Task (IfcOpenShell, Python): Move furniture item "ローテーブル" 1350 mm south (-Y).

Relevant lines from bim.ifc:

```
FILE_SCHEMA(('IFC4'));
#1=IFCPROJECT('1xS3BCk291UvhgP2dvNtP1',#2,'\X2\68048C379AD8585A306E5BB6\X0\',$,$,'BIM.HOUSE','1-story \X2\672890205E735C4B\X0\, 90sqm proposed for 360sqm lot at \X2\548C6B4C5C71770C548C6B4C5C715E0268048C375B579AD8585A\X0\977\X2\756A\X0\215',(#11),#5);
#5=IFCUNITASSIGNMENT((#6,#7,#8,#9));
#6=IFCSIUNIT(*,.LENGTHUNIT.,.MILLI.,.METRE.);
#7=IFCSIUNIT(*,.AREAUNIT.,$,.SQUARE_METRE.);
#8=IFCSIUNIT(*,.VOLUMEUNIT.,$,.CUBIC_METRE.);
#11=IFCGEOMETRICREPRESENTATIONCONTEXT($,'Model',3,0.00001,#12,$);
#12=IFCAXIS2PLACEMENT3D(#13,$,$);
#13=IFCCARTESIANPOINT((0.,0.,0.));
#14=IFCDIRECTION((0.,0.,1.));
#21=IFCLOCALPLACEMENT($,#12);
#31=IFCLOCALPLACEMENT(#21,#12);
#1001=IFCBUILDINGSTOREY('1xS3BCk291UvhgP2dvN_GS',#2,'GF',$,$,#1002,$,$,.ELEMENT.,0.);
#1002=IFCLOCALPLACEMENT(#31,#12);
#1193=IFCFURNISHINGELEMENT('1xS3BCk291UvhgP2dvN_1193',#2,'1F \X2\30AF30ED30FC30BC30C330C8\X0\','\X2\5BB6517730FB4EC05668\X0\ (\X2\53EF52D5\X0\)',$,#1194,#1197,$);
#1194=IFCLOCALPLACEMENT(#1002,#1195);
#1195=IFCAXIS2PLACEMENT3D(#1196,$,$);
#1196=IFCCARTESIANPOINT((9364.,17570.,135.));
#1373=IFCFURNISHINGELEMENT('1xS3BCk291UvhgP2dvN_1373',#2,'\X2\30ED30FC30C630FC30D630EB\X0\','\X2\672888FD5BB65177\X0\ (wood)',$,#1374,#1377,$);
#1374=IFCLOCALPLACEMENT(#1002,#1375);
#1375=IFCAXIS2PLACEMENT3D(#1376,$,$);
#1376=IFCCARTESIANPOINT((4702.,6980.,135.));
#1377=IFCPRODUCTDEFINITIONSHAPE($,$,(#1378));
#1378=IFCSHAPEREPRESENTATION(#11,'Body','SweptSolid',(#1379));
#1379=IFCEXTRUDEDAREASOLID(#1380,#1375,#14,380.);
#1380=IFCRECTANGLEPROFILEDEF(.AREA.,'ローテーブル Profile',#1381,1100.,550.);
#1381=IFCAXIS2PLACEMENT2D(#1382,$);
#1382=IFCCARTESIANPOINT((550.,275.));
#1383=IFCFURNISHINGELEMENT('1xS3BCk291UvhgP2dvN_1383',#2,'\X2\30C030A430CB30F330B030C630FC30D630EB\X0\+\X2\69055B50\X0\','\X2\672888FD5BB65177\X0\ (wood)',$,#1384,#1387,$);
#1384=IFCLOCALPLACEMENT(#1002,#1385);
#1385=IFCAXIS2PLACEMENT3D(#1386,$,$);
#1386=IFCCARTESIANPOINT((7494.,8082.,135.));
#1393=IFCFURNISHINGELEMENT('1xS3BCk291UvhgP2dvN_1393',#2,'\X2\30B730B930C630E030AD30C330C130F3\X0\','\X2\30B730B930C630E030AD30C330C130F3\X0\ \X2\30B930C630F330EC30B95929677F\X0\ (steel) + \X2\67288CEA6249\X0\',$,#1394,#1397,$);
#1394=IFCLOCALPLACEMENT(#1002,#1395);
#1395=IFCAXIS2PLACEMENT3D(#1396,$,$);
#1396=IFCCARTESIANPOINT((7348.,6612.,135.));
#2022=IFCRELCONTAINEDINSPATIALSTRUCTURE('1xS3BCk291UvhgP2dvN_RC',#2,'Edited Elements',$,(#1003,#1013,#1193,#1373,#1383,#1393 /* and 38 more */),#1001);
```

```python
import ifcopenshell
import ifcopenshell.api.geometry
import ifcopenshell.util.placement
import ifcopenshell.util.unit

model = ifcopenshell.open("bim.ifc")
unit_scale = ifcopenshell.util.unit.calculate_unit_scale(model)

item = model.by_guid("1xS3BCk291UvhgP2dvN_1373")
matrix = ifcopenshell.util.placement.get_local_placement(item.ObjectPlacement)
matrix[1, 3] -= 1.35 / unit_scale
ifcopenshell.api.geometry.edit_object_placement(model, product=item, matrix=matrix, is_si=False)

print(ifcopenshell.util.placement.get_local_placement(item.ObjectPlacement).round(3) + 0.0)

model.write("bim_edited.ifc")
```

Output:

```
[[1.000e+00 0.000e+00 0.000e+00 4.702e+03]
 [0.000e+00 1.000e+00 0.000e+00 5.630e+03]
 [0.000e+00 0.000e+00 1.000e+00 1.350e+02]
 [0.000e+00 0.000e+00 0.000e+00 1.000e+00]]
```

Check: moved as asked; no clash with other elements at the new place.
